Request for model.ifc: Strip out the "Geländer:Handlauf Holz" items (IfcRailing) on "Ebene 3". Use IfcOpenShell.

First a look at what the model holds.

```python
import ifcopenshell
import ifcopenshell.util.element

model = ifcopenshell.open("model.ifc")
print(model.schema)
storey = next(s for s in model.by_type("IfcBuildingStorey") if s.Name == "Ebene 3")
railings = [e for e in ifcopenshell.util.element.get_decomposition(storey) if e.is_a("IfcRailing")]
seen = {}
for e in railings:
    element_type = ifcopenshell.util.element.get_type(e)
    name = element_type.Name if element_type not in (None, e) else None
    seen[name] = seen.get(name, 0) + 1
for name, count in sorted(seen.items(), key=str):
    print(count, "x", name)
```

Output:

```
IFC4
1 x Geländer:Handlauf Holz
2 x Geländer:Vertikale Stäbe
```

```python
import ifcopenshell
import ifcopenshell.api.root
import ifcopenshell.util.element

model = ifcopenshell.open("model.ifc")

storey = next(s for s in model.by_type("IfcBuildingStorey") if s.Name == "Ebene 3")
railings = [e for e in ifcopenshell.util.element.get_decomposition(storey) if e.is_a("IfcRailing")]
targets = [e for e in railings if (t := ifcopenshell.util.element.get_type(e)) not in (None, e) and t.Name == "Geländer:Handlauf Holz"]

for e in targets:
    ifcopenshell.api.root.remove_product(model, product=e)
print(len(targets), "removed")

model.write("model-out.ifc")
```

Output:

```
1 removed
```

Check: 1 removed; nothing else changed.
